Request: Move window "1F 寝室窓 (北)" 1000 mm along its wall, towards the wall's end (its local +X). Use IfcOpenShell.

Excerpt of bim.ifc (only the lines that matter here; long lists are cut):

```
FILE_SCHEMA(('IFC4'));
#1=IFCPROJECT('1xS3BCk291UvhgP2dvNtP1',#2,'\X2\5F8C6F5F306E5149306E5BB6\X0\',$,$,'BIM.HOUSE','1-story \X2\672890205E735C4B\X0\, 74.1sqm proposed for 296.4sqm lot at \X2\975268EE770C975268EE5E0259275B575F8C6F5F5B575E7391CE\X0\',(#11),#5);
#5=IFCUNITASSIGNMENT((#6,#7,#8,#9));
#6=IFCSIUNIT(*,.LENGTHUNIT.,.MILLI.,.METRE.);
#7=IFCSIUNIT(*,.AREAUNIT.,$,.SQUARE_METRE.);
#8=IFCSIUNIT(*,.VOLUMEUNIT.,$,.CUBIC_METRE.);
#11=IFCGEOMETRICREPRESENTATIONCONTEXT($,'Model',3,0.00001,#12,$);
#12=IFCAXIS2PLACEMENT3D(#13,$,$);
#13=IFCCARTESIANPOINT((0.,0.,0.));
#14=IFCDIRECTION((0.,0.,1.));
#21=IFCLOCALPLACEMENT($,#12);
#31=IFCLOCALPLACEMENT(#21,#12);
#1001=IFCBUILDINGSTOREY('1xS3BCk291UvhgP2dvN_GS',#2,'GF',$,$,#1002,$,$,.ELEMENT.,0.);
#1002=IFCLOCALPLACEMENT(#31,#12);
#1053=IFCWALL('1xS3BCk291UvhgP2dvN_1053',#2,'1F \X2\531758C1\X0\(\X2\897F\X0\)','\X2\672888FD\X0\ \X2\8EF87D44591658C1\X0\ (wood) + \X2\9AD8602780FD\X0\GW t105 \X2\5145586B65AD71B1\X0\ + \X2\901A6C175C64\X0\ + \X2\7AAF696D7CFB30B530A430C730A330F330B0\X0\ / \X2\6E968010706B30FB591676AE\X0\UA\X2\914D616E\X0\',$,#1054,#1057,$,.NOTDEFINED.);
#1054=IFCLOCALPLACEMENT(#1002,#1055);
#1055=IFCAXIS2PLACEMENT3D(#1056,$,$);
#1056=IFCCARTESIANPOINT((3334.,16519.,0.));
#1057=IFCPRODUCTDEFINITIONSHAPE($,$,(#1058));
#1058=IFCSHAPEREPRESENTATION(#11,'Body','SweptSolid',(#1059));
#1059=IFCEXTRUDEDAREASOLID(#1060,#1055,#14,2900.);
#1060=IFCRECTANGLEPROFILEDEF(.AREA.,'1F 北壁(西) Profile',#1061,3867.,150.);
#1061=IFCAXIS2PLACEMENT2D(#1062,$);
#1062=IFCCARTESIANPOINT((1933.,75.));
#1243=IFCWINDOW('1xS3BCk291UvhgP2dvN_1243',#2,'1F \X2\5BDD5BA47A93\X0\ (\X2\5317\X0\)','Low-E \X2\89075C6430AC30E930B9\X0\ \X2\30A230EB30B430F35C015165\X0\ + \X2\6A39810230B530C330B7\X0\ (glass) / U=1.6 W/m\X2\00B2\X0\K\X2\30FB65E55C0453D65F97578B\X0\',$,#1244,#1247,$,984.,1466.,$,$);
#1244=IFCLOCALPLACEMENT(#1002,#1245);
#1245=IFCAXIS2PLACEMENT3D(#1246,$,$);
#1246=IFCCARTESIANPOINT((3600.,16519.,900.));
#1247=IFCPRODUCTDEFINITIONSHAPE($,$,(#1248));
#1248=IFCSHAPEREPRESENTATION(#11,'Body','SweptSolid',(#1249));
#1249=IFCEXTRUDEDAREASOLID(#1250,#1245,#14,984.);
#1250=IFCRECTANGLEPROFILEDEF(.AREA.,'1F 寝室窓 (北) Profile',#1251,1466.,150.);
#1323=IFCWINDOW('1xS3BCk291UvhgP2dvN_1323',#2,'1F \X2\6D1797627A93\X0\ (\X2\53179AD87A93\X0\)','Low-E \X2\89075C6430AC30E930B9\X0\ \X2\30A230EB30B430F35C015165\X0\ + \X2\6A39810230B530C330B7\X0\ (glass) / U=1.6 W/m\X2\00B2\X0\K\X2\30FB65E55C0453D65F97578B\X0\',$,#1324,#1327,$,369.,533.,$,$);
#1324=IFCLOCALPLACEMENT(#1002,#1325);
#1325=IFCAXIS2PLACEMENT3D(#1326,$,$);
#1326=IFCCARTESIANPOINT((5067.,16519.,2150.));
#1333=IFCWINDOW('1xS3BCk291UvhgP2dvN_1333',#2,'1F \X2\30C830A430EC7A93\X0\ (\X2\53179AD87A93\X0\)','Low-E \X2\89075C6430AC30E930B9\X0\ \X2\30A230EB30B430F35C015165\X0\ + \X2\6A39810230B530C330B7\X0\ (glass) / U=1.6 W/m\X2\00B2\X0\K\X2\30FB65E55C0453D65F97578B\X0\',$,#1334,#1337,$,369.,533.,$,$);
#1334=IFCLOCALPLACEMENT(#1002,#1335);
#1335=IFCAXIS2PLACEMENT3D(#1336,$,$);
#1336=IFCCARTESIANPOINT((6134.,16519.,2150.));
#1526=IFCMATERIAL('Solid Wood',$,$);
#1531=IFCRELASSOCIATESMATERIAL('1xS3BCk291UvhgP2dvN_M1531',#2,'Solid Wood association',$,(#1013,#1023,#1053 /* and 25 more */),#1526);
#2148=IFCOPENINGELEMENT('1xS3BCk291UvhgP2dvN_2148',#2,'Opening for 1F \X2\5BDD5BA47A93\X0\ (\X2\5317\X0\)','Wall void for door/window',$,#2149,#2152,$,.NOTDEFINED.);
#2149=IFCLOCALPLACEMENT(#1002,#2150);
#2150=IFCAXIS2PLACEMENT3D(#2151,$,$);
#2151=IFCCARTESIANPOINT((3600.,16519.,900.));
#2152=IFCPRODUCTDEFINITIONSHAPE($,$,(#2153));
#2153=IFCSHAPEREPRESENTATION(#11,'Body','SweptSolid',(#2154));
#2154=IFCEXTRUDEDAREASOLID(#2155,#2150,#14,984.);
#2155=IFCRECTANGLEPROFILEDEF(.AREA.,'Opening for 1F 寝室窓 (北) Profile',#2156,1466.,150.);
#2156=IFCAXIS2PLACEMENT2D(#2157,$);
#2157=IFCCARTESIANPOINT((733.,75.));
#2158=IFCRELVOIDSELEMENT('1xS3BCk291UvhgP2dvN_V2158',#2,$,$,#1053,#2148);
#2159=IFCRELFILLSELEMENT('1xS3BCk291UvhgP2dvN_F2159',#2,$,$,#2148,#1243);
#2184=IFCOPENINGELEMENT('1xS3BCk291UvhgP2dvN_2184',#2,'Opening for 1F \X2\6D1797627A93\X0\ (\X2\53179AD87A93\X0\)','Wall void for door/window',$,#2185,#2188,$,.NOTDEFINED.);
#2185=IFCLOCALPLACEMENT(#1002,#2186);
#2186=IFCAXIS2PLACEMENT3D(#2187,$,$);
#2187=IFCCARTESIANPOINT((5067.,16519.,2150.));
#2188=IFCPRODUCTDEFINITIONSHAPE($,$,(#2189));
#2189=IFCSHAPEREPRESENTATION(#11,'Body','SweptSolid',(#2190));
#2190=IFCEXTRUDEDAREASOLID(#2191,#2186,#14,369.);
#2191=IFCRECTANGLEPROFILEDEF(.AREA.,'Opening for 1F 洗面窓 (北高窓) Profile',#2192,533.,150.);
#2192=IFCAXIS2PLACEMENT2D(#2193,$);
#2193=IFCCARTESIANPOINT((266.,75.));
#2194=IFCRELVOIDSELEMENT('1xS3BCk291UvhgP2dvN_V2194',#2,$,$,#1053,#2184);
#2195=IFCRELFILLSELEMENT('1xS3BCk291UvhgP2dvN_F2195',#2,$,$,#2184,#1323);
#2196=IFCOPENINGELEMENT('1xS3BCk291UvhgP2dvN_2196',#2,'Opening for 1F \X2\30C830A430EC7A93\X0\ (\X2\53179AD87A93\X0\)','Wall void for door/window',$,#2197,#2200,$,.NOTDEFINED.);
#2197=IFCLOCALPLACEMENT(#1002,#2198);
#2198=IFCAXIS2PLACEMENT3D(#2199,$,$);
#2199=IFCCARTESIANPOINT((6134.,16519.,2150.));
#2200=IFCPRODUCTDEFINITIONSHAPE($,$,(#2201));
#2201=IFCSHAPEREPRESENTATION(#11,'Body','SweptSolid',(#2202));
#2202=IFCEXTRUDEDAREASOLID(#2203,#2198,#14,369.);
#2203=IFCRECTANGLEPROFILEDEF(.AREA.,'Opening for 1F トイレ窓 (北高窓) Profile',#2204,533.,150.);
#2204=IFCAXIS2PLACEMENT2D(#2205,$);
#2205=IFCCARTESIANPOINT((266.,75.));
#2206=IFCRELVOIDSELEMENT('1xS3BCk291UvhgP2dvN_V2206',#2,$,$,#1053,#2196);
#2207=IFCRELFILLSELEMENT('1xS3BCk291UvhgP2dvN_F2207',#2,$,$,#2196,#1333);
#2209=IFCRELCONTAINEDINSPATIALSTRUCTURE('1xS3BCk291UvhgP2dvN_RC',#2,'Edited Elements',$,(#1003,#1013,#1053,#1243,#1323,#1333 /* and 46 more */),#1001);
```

```python
import ifcopenshell
import ifcopenshell.api.geometry
import ifcopenshell.util.placement

model = ifcopenshell.open("bim.ifc")

window = model.by_id(1243)
opening = window.FillsVoids[0].RelatingOpeningElement
wall = opening.VoidsElements[0].RelatingBuildingElement

wall_matrix = ifcopenshell.util.placement.get_local_placement(wall.ObjectPlacement)
shift = wall_matrix[:3, 0] * 1000.0
before = ifcopenshell.util.placement.get_local_placement(window.ObjectPlacement)[:3, 3].copy()

# The window is not placed relative to its opening, so move both.
for product in (opening, window):
    matrix = ifcopenshell.util.placement.get_local_placement(product.ObjectPlacement)
    matrix[:3, 3] += shift
    ifcopenshell.api.geometry.edit_object_placement(model, product=product, matrix=matrix, is_si=False)

after = ifcopenshell.util.placement.get_local_placement(window.ObjectPlacement)[:3, 3]
print("window moved by", (after - before).round(3) + 0.0)

model.write("bim-out.ifc")
```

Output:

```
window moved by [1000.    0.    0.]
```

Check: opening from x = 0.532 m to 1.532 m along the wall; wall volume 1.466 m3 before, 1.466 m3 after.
